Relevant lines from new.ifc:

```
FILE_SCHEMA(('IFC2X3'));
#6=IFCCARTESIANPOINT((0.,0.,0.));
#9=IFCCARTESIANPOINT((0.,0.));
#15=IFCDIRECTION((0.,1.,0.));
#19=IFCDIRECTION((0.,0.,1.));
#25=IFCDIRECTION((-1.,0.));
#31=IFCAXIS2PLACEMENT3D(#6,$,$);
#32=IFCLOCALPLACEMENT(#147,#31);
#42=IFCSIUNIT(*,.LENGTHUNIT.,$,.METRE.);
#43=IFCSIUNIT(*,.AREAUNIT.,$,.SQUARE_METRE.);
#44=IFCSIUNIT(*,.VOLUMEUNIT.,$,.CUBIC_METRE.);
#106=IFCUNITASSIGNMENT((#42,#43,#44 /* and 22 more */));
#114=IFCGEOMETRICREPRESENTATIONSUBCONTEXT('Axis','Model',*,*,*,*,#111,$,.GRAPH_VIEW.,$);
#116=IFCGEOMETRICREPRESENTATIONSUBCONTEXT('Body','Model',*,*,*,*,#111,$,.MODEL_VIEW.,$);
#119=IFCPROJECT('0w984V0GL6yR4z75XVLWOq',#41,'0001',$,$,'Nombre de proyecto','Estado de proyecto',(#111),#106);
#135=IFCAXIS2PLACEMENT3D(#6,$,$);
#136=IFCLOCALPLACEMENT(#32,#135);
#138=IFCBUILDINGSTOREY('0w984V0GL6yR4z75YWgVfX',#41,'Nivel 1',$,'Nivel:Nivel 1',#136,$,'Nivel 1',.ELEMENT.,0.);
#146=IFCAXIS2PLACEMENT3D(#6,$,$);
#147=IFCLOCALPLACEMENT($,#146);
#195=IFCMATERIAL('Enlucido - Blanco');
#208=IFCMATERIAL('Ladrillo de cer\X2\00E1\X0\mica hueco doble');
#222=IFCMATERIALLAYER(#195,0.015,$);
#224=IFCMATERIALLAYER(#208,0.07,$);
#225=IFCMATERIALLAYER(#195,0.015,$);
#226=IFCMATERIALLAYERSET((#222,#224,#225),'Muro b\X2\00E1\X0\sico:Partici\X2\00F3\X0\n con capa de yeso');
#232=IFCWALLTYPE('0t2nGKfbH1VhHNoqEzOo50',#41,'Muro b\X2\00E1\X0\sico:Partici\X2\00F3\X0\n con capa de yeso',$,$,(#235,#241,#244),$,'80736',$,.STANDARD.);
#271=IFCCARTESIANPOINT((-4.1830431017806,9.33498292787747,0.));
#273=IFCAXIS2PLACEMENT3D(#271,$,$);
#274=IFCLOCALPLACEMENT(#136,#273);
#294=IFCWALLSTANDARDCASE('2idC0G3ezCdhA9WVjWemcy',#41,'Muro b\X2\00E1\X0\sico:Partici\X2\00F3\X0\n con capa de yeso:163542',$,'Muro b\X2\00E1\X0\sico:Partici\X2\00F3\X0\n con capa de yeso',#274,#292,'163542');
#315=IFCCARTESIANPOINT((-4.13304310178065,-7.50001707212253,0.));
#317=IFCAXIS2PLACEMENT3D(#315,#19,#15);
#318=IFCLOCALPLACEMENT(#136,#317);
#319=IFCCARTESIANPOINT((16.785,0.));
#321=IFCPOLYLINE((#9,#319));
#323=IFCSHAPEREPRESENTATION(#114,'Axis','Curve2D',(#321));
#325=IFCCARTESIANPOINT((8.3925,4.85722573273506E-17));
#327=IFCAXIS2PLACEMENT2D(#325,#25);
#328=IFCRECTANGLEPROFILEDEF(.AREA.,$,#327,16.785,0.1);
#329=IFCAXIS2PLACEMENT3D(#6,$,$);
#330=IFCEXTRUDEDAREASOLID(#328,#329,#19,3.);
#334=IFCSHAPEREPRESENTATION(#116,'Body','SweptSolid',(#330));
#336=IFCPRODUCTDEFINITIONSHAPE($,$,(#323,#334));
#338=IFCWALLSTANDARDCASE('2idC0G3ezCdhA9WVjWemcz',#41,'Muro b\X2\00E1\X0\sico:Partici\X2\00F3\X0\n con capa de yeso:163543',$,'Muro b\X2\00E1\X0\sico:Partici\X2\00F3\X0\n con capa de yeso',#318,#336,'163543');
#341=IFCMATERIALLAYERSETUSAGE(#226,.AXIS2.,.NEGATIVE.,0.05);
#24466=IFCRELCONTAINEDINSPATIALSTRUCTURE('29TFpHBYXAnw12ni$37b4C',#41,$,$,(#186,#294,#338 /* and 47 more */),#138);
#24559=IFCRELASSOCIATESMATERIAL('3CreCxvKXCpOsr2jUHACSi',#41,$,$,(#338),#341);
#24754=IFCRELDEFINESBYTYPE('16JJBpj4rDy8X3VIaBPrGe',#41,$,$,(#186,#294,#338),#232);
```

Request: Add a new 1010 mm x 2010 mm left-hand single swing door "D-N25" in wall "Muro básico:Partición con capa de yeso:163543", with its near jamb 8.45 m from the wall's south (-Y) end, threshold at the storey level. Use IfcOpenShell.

```python
import numpy as np
import ifcopenshell
import ifcopenshell.api.feature
import ifcopenshell.api.geometry
import ifcopenshell.api.root
import ifcopenshell.api.spatial
import ifcopenshell.api.type
import ifcopenshell.geom
import ifcopenshell.util.element
import ifcopenshell.util.placement
import ifcopenshell.util.representation
import ifcopenshell.util.shape
import ifcopenshell.util.unit

model = ifcopenshell.open("new.ifc")
unit_scale = ifcopenshell.util.unit.calculate_unit_scale(model)
settings = ifcopenshell.geom.settings()


def volume(element):
    """Net volume in cubic metres, openings subtracted."""
    shape = ifcopenshell.geom.create_shape(settings, element)
    return ifcopenshell.util.shape.get_volume(shape.geometry)


wall = model.by_guid("2idC0G3ezCdhA9WVjWemcz")
storey = ifcopenshell.util.element.get_container(wall, ifc_class="IfcBuildingStorey")
context = ifcopenshell.util.representation.get_context(model, "Model", "Body", "MODEL_VIEW")
before = volume(wall)

width, height, from_end, sill = 1.01, 2.01, 8.45, 0.0  # metres

# The wall runs along its own X axis, and the end named is its -X end.
wall_shape = ifcopenshell.geom.create_shape(settings, wall)
x, y, z = ifcopenshell.util.shape.get_vertices(wall_shape.geometry).T
start = x.min() + from_end
face, thickness = float(y.min()), float(y.max() - y.min())
wall_matrix = ifcopenshell.util.placement.get_local_placement(wall.ObjectPlacement)
level = ifcopenshell.util.placement.get_local_placement(storey.ObjectPlacement)[2, 3]


def in_wall(x, y):
    """Placement at x, y metres in the wall's axes, at sill height."""
    matrix = wall_matrix.copy()
    matrix[:, 3] = wall_matrix @ np.array([x / unit_scale, y / unit_scale, 0.0, 1.0])
    matrix[2, 3] = level + sill / unit_scale
    return matrix


# Opening: a box that overshoots both wall faces by 50 mm.
opening = ifcopenshell.api.root.create_entity(model, ifc_class="IfcOpeningElement")
box = ifcopenshell.api.geometry.add_wall_representation(
    model, context=context, length=width, height=height, thickness=thickness + 0.1
)
ifcopenshell.api.geometry.assign_representation(model, product=opening, representation=box)
ifcopenshell.api.geometry.edit_object_placement(model, product=opening, matrix=in_wall(start, face - 0.05), is_si=False)
ifcopenshell.api.feature.add_feature(model, feature=opening, element=wall)

door = ifcopenshell.api.root.create_entity(model, ifc_class="IfcDoor", name="D-N25")
door.OverallWidth, door.OverallHeight = width / unit_scale, height / unit_scale
body = ifcopenshell.api.geometry.add_door_representation(
    model,
    context=context,
    overall_width=door.OverallWidth,
    overall_height=door.OverallHeight,
    operation_type="SINGLE_SWING_LEFT",
    lining_properties={"LiningDepth": thickness / unit_scale, "ThresholdDepth": thickness / unit_scale},
)
ifcopenshell.api.geometry.assign_representation(model, product=door, representation=body)
ifcopenshell.api.spatial.assign_container(model, products=[door], relating_structure=storey)
fills = ifcopenshell.api.feature.add_filling(model, opening=opening, element=door)
fills.OwnerHistory = door.OwnerHistory  # required in IFC2X3

# IFC2X3 keeps the operation on the door style.
style = ifcopenshell.api.root.create_entity(model, ifc_class="IfcDoorStyle", name="D-N25")
style.OperationType, style.ConstructionType = "SINGLE_SWING_LEFT", "NOTDEFINED"
style.ParameterTakesPrecedence = style.Sizeable = False
ifcopenshell.api.type.assign_type(model, related_objects=[door], relating_type=style)

# The lining spans the wall, so the door starts at the wall face.
ifcopenshell.api.geometry.edit_object_placement(model, product=door, matrix=in_wall(start, face), is_si=False)

after = volume(wall)

print(f"wall volume {before:.3f} -> {after:.3f} m3")

model.write("new_rev.ifc")
```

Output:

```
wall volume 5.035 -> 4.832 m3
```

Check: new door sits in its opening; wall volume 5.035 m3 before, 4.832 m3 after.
